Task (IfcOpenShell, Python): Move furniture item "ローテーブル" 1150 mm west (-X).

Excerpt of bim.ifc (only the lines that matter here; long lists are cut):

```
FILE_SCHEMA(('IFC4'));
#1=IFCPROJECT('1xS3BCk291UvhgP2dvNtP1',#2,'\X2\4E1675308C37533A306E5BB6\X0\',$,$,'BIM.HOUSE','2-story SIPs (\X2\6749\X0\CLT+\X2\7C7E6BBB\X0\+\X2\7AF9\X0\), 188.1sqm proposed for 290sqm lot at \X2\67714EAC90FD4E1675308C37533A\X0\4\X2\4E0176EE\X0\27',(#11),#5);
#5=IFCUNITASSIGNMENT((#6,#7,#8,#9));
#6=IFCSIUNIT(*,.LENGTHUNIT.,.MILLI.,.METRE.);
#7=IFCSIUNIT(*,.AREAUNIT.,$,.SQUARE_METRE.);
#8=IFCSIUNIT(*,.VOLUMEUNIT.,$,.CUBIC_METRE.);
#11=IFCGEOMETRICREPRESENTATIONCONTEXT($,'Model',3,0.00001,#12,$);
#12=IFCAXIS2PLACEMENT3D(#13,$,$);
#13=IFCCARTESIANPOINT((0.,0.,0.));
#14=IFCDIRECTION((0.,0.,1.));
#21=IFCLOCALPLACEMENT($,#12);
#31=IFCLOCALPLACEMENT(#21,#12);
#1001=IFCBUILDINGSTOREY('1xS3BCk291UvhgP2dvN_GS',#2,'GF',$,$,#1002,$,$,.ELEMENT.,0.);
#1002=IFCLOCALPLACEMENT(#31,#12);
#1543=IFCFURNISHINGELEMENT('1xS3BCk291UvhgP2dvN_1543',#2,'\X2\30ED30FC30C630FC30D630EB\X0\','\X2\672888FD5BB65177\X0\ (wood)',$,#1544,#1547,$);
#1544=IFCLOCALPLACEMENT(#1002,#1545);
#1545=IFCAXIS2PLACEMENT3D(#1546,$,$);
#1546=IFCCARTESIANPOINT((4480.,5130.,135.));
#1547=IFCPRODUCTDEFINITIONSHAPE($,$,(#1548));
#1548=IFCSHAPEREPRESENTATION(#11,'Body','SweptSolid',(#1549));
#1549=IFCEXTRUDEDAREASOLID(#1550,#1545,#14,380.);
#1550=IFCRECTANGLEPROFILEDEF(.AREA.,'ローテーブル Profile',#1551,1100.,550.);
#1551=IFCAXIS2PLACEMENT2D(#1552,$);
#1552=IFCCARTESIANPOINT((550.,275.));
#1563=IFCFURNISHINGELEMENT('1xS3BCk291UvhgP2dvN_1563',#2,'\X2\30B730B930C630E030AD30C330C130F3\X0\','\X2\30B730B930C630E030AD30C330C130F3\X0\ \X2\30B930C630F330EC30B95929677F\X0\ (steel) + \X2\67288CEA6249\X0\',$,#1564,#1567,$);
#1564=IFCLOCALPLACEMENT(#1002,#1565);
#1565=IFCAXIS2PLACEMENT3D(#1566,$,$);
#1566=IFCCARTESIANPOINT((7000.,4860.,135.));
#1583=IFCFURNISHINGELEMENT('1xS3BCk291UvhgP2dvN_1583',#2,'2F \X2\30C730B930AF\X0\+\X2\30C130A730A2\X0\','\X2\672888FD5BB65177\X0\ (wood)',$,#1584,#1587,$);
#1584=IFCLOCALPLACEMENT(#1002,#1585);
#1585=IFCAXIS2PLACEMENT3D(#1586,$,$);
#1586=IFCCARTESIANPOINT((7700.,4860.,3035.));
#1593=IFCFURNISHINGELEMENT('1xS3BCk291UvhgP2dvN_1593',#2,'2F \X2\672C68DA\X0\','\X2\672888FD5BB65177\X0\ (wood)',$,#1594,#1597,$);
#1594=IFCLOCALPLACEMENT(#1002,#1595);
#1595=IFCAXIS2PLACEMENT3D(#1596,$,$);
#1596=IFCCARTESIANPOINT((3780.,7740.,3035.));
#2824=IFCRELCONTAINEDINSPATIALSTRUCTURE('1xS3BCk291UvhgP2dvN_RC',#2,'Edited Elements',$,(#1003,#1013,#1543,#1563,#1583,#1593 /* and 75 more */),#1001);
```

```python
import ifcopenshell
import ifcopenshell.api.geometry
import ifcopenshell.util.placement

model = ifcopenshell.open("bim.ifc")

item = model.by_id(1543)
matrix = ifcopenshell.util.placement.get_local_placement(item.ObjectPlacement)
matrix[0, 3] -= 1150.0
ifcopenshell.api.geometry.edit_object_placement(model, product=item, matrix=matrix, is_si=False)

print(ifcopenshell.util.placement.get_local_placement(item.ObjectPlacement).round(3) + 0.0)

model.write("bim_updated.ifc")
```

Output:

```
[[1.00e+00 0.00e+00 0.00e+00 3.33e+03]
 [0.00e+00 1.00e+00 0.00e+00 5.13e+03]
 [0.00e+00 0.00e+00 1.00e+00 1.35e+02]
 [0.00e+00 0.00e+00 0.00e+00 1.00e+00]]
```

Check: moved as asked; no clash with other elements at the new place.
